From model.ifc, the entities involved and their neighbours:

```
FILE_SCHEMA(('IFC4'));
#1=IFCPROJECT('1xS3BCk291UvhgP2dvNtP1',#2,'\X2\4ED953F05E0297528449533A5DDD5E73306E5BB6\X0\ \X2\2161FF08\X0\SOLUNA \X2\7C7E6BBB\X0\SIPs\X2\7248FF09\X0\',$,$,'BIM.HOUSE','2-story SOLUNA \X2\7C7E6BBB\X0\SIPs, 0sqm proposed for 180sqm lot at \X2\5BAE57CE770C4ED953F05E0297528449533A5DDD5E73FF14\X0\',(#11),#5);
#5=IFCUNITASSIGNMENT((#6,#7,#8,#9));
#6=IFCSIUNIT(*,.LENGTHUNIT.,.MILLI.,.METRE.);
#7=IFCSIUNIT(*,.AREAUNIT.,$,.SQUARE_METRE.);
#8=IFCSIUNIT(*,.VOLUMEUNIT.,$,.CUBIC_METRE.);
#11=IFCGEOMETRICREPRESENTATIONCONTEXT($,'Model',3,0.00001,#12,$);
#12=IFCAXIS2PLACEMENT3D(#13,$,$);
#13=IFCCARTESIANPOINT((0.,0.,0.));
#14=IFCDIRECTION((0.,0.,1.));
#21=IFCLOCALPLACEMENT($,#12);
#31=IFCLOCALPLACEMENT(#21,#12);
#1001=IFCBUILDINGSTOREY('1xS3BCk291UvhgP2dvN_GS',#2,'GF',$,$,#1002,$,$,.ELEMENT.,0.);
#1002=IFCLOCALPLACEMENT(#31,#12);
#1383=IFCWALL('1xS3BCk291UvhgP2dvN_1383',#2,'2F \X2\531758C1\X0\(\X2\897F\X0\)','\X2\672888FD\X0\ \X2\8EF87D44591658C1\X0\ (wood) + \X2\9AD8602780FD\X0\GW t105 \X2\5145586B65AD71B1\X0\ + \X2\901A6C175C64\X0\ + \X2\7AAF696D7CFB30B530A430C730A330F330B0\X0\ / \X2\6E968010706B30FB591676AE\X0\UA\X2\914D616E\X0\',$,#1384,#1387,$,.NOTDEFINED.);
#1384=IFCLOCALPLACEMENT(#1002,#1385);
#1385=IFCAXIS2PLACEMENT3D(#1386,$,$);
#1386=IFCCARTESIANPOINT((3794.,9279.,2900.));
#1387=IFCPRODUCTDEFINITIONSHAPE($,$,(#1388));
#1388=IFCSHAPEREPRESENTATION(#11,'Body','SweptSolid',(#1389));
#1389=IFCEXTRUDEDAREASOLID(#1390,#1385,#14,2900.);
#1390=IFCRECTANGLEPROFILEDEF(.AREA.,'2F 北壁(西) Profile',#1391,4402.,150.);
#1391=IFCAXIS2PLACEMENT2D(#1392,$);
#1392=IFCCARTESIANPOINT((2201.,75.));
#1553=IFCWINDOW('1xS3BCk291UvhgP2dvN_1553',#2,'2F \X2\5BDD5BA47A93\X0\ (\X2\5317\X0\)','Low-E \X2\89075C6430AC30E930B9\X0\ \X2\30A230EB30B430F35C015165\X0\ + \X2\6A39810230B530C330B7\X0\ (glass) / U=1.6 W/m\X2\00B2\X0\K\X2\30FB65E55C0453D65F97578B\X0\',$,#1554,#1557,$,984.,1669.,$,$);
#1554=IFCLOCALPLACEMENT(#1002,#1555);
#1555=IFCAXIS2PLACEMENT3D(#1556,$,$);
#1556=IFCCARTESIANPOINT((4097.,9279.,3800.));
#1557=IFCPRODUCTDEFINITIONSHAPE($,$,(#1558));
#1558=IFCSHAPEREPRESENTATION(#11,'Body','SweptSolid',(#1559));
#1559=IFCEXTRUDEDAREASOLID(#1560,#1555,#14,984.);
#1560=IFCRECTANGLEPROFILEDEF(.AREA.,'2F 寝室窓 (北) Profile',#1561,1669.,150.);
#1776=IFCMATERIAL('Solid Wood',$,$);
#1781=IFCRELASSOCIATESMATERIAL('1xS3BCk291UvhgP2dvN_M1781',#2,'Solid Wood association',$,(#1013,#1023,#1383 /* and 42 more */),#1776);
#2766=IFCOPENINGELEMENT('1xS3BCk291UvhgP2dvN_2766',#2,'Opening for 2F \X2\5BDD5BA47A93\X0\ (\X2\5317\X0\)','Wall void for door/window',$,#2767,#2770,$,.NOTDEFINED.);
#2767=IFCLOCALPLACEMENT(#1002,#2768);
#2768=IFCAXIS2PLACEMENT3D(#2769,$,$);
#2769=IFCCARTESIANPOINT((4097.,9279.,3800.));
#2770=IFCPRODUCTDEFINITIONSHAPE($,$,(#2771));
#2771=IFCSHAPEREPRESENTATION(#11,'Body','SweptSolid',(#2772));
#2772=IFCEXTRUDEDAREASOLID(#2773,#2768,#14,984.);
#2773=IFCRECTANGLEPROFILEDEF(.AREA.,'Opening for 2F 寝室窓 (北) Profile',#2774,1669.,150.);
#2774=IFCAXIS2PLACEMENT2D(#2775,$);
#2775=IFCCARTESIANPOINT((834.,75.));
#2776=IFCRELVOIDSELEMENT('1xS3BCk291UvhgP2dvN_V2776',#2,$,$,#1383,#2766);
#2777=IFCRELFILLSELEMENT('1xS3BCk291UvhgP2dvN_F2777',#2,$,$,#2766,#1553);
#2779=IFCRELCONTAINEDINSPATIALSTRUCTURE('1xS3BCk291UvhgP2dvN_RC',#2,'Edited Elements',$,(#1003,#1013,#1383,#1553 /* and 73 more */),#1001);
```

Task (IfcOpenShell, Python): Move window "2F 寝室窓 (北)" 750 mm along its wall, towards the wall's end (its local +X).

```python
import ifcopenshell
import ifcopenshell.api.geometry
import ifcopenshell.util.placement
import ifcopenshell.util.unit

model = ifcopenshell.open("model.ifc")
unit_scale = ifcopenshell.util.unit.calculate_unit_scale(model)

window = model.by_id(1553)
opening = window.FillsVoids[0].RelatingOpeningElement
wall = opening.VoidsElements[0].RelatingBuildingElement

wall_matrix = ifcopenshell.util.placement.get_local_placement(wall.ObjectPlacement)
shift = wall_matrix[:3, 0] * 0.75 / unit_scale
before = ifcopenshell.util.placement.get_local_placement(window.ObjectPlacement)[:3, 3].copy()

# The window is not placed relative to its opening, so move both.
for product in (opening, window):
    matrix = ifcopenshell.util.placement.get_local_placement(product.ObjectPlacement)
    matrix[:3, 3] += shift
    ifcopenshell.api.geometry.edit_object_placement(model, product=product, matrix=matrix, is_si=False)

after = ifcopenshell.util.placement.get_local_placement(window.ObjectPlacement)[:3, 3]
print("window moved by", (after - before).round(3) + 0.0)

model.write("model_edited.ifc")
```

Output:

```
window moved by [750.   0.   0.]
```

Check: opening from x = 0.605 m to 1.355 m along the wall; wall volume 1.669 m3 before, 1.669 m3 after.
